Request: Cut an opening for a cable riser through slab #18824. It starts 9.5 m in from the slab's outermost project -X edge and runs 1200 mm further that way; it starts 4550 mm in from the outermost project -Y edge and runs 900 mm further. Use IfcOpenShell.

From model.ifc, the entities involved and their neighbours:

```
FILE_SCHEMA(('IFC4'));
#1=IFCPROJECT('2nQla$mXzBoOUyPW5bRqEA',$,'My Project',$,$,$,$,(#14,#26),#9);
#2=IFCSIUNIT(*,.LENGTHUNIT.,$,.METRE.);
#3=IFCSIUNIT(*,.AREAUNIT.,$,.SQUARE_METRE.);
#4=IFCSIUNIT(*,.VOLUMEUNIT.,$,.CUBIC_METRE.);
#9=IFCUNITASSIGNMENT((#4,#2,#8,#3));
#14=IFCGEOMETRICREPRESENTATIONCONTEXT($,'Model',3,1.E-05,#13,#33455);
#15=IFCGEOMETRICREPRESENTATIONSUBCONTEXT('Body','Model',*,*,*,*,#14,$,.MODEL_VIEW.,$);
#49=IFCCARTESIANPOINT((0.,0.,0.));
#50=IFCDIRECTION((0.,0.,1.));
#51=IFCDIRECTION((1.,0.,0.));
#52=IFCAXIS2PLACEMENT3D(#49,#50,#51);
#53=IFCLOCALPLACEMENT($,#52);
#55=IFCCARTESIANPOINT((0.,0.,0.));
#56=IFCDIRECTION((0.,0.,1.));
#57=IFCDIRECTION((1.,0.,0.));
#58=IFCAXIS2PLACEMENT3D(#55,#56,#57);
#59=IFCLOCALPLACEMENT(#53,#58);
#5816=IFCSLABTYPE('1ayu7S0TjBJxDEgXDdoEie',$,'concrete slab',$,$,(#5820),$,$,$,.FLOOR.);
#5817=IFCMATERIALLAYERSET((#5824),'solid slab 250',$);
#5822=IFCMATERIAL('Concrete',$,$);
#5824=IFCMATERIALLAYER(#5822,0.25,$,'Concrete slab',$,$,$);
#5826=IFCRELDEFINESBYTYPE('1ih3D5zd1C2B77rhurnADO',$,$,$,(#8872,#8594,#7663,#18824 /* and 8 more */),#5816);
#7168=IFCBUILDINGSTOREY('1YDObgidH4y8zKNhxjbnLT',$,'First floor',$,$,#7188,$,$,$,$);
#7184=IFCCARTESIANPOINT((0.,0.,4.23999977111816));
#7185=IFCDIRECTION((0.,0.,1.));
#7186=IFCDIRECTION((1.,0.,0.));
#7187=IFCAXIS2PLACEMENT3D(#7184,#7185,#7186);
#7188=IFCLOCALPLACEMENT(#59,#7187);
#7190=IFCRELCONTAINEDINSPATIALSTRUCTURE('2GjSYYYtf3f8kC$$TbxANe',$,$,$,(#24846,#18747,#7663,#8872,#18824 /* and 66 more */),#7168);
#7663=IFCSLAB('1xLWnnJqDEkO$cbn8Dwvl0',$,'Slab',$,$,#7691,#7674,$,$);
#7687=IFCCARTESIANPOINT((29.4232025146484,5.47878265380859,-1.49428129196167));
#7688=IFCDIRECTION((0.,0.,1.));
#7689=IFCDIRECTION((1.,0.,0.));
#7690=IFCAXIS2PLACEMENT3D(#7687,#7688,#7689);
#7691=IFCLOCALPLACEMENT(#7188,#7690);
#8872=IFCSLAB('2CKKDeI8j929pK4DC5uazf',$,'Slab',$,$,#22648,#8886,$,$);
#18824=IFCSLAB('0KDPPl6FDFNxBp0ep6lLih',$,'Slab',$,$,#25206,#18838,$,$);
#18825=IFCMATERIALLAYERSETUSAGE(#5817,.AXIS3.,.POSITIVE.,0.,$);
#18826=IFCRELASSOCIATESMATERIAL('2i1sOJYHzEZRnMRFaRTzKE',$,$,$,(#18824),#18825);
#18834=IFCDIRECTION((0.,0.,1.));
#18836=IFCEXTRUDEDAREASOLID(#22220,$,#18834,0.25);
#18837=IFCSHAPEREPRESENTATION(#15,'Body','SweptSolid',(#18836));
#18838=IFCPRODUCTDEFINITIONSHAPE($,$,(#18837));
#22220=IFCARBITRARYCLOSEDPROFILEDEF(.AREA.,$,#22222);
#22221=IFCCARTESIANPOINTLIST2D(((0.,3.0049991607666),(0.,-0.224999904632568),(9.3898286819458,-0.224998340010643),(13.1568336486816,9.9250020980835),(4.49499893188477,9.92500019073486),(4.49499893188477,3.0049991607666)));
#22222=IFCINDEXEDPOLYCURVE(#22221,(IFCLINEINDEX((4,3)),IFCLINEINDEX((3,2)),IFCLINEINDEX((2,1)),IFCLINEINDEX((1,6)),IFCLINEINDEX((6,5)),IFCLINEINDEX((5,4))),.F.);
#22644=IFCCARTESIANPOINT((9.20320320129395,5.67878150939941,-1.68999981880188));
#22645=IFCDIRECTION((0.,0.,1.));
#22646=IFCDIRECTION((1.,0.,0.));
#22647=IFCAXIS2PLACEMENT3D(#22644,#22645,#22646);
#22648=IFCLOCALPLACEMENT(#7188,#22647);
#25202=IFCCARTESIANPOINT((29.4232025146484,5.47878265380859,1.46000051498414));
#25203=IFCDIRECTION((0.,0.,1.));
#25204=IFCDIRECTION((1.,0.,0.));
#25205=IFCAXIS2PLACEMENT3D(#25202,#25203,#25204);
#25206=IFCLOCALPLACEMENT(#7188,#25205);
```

```python
import numpy as np
import ifcopenshell
import ifcopenshell.api.feature
import ifcopenshell.api.geometry
import ifcopenshell.api.root
import ifcopenshell.geom
import ifcopenshell.util.placement
import ifcopenshell.util.representation
import ifcopenshell.util.shape
import ifcopenshell.util.unit

model = ifcopenshell.open("model.ifc")
unit_scale = ifcopenshell.util.unit.calculate_unit_scale(model)
settings = ifcopenshell.geom.settings()


def volume(element):
    """Net volume in cubic metres, openings subtracted."""
    shape = ifcopenshell.geom.create_shape(settings, element)
    return ifcopenshell.util.shape.get_volume(shape.geometry)


slab = model.by_id(18824)
before = volume(slab)

# Extent in the slab's own axes, in metres. The edges named are its -X and -Y sides.
slab_shape = ifcopenshell.geom.create_shape(settings, slab)
vertices = ifcopenshell.util.shape.get_vertices(slab_shape.geometry)
x_min, y_min, bottom = vertices.min(axis=0)
top = vertices[:, 2].max()

opening = ifcopenshell.api.root.create_entity(model, ifc_class="IfcOpeningElement", name="Cable riser opening", predefined_type="OPENING")
context = ifcopenshell.util.representation.get_context(model, "Model", "Body", "MODEL_VIEW")
width, depth = 1.2, 0.9
outline = [(0.0, 0.0), (width, 0.0), (width, depth), (0.0, depth), (0.0, 0.0)]
# Overshoot both faces by 50 mm so the cut is clean.
shape = ifcopenshell.api.geometry.add_slab_representation(
    model, context=context, depth=top - bottom + 0.1, polyline=outline
)
ifcopenshell.api.geometry.assign_representation(model, product=opening, representation=shape)

matrix = ifcopenshell.util.placement.get_local_placement(slab.ObjectPlacement)
matrix[:, 3] = matrix @ np.append(np.array([x_min + 9.5, y_min + 4.55, bottom - 0.05]) / unit_scale, 1.0)
ifcopenshell.api.geometry.edit_object_placement(model, product=opening, matrix=matrix, is_si=False)
ifcopenshell.api.feature.add_feature(model, feature=opening, element=slab)

after = volume(slab)

print(f"slab volume {before:.3f} -> {after:.3f} m3")

model.write("model_edited.ifc")
```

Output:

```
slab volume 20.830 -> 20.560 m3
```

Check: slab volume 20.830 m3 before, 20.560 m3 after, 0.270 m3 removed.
